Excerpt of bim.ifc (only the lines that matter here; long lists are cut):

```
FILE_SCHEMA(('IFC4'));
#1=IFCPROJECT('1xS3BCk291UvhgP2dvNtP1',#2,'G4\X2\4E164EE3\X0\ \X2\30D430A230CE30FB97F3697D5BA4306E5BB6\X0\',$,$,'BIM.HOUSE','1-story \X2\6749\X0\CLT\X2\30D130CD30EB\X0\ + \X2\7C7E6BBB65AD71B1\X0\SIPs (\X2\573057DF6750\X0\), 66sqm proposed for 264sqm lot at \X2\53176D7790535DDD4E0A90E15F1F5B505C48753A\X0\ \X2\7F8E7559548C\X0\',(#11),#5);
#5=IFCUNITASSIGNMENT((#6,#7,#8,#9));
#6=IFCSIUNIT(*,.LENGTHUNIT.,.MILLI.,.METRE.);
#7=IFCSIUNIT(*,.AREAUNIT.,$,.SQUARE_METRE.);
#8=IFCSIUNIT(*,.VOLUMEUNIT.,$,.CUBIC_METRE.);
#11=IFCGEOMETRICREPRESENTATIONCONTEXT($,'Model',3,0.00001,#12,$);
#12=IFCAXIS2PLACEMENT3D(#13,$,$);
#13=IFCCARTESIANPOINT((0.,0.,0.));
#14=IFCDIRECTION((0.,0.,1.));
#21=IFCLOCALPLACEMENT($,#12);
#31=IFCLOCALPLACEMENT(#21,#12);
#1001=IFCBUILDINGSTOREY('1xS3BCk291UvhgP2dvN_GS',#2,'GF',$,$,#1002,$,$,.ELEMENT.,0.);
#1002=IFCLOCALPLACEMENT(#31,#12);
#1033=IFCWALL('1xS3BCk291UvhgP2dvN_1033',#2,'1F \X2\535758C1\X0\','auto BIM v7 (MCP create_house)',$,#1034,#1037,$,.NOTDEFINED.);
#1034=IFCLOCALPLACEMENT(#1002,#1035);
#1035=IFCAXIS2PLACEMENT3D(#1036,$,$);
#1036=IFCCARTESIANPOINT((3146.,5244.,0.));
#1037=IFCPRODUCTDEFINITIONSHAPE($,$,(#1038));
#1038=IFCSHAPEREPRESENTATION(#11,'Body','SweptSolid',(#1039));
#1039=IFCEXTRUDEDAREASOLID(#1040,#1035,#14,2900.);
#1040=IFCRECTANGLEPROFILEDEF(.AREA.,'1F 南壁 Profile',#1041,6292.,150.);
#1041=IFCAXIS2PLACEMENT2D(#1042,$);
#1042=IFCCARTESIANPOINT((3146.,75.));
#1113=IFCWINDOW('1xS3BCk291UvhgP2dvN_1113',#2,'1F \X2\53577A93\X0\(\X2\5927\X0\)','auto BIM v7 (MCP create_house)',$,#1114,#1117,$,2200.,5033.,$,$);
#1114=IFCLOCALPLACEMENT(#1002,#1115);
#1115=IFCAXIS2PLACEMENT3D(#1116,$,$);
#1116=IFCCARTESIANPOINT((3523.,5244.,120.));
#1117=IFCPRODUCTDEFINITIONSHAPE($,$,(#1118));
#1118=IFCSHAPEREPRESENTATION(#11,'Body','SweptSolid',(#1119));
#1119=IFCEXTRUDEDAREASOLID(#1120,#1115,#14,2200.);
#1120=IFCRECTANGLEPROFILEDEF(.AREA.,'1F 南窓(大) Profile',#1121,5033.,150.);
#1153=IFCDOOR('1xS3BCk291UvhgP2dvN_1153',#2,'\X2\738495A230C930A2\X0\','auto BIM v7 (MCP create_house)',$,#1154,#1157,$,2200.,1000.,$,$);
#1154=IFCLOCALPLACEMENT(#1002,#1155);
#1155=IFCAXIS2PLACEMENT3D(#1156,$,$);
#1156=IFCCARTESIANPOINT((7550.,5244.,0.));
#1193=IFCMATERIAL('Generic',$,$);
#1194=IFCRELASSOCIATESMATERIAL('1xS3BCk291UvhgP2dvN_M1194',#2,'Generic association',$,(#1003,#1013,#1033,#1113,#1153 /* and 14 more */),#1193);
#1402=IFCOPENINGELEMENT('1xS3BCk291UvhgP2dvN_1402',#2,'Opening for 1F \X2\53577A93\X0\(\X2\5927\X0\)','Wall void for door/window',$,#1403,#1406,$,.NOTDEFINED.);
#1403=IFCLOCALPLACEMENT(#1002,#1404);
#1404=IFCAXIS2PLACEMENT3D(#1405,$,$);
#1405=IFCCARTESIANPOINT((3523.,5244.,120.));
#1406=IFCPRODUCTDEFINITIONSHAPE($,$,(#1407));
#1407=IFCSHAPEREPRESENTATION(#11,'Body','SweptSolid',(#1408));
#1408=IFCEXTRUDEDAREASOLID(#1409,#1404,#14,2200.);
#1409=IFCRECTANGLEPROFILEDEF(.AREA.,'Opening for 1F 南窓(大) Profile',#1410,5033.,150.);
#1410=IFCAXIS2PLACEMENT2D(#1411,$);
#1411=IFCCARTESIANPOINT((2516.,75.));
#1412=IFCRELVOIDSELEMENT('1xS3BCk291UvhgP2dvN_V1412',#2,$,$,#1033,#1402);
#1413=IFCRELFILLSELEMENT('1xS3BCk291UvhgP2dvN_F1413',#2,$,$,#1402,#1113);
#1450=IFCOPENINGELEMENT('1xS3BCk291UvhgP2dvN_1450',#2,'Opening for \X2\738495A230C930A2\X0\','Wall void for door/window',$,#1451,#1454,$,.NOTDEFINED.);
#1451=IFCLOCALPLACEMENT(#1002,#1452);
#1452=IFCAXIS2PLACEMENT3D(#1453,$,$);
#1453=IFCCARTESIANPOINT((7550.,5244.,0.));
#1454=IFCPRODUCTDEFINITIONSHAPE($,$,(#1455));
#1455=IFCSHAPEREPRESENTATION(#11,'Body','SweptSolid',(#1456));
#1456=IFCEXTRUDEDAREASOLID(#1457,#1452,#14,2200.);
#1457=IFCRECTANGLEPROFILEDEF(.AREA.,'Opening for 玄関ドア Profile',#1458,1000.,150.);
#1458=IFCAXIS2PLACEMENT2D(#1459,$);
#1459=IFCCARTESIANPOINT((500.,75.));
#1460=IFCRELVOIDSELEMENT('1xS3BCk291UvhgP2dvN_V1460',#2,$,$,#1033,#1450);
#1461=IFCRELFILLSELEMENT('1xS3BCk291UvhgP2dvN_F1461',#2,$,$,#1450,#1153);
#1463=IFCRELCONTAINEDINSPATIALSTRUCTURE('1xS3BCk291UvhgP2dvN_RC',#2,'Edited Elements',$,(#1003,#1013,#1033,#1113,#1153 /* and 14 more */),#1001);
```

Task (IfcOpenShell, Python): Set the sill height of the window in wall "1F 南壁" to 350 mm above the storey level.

```python
import numpy as np
import ifcopenshell
import ifcopenshell.api.geometry
import ifcopenshell.geom
import ifcopenshell.util.element
import ifcopenshell.util.placement
import ifcopenshell.util.shape
import ifcopenshell.util.unit

model = ifcopenshell.open("bim.ifc")
unit_scale = ifcopenshell.util.unit.calculate_unit_scale(model)

window = model.by_id(1113)
opening = window.FillsVoids[0].RelatingOpeningElement
storey = ifcopenshell.util.element.get_container(window, ifc_class="IfcBuildingStorey")
level = ifcopenshell.util.placement.get_local_placement(storey.ObjectPlacement)[2, 3]

# The opening's origin need not be at the sill, so measure its lowest point.
shape = ifcopenshell.geom.create_shape(ifcopenshell.geom.settings(), opening)
bottom = ifcopenshell.util.shape.get_shape_bottom_elevation(shape, shape.geometry) / unit_scale
dz = level + 0.35 / unit_scale - bottom

shift = np.array([0.0, 0.0, dz])
# The window is not placed relative to its opening, so move both.
for product in (opening, window):
    matrix = ifcopenshell.util.placement.get_local_placement(product.ObjectPlacement)
    matrix[:3, 3] += shift
    ifcopenshell.api.geometry.edit_object_placement(model, product=product, matrix=matrix, is_si=False)

print(f"moved by {dz * unit_scale:+.3f} m")

model.write("bim_updated.ifc")
```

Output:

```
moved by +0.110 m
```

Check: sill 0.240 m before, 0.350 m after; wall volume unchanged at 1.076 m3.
